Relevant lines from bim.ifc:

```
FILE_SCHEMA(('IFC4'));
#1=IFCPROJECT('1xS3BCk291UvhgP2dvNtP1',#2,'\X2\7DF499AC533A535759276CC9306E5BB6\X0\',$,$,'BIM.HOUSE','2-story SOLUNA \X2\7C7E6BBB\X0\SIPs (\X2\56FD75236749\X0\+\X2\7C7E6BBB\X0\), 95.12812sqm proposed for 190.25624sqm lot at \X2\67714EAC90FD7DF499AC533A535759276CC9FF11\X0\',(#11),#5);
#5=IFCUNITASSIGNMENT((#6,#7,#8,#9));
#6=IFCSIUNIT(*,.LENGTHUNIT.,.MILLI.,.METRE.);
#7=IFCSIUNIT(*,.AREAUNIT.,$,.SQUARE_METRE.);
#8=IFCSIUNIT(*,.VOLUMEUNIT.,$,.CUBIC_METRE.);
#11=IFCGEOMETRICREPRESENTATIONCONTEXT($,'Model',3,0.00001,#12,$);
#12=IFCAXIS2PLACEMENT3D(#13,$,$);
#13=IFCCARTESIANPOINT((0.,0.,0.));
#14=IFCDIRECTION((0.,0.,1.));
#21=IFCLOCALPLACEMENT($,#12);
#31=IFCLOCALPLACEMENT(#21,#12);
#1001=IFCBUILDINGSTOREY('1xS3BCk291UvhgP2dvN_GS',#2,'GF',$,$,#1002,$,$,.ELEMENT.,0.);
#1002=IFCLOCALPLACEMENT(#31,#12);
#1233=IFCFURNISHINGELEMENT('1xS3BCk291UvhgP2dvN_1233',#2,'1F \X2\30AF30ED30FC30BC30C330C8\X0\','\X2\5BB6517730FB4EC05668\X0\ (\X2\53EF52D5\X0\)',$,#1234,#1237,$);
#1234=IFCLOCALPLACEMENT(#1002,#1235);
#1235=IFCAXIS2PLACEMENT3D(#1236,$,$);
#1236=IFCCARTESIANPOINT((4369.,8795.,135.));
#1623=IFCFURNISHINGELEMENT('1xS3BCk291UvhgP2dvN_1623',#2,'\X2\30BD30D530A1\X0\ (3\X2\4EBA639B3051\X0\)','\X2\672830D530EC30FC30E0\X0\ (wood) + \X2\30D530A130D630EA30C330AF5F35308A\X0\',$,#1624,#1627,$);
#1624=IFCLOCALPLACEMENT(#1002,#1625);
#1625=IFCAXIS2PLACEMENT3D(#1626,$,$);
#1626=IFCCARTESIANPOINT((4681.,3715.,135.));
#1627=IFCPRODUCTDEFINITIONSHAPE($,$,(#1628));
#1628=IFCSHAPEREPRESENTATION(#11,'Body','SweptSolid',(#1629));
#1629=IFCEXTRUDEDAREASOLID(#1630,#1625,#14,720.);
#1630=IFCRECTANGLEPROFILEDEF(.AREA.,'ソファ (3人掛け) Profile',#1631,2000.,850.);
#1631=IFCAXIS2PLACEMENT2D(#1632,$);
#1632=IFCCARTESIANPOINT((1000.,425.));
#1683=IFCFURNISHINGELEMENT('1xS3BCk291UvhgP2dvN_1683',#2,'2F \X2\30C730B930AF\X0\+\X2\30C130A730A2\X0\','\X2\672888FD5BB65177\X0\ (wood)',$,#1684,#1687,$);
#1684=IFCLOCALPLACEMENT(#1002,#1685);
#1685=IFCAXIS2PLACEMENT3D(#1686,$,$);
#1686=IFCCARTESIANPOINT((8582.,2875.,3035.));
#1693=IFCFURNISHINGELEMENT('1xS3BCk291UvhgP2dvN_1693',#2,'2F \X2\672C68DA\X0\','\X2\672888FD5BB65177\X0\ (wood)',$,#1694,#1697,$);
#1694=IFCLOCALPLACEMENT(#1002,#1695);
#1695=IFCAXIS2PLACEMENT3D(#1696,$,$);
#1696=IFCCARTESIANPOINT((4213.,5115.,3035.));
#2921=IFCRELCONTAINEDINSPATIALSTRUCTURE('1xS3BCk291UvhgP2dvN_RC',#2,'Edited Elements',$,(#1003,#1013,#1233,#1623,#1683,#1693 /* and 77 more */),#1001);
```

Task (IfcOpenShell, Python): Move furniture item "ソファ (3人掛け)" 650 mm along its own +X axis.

```python
import ifcopenshell
import ifcopenshell.api.geometry
import ifcopenshell.util.placement

model = ifcopenshell.open("bim.ifc")

item = model.by_guid("1xS3BCk291UvhgP2dvN_1623")
matrix = ifcopenshell.util.placement.get_local_placement(item.ObjectPlacement)
matrix[:3, 3] += matrix[:3, 0] * 650.0
ifcopenshell.api.geometry.edit_object_placement(model, product=item, matrix=matrix, is_si=False)

print(ifcopenshell.util.placement.get_local_placement(item.ObjectPlacement).round(3) + 0.0)

model.write("bim_edited.ifc")
```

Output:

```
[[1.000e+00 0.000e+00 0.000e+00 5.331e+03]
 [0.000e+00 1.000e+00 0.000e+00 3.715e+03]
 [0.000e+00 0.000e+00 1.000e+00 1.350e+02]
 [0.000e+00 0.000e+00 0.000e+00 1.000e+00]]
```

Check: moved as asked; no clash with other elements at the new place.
